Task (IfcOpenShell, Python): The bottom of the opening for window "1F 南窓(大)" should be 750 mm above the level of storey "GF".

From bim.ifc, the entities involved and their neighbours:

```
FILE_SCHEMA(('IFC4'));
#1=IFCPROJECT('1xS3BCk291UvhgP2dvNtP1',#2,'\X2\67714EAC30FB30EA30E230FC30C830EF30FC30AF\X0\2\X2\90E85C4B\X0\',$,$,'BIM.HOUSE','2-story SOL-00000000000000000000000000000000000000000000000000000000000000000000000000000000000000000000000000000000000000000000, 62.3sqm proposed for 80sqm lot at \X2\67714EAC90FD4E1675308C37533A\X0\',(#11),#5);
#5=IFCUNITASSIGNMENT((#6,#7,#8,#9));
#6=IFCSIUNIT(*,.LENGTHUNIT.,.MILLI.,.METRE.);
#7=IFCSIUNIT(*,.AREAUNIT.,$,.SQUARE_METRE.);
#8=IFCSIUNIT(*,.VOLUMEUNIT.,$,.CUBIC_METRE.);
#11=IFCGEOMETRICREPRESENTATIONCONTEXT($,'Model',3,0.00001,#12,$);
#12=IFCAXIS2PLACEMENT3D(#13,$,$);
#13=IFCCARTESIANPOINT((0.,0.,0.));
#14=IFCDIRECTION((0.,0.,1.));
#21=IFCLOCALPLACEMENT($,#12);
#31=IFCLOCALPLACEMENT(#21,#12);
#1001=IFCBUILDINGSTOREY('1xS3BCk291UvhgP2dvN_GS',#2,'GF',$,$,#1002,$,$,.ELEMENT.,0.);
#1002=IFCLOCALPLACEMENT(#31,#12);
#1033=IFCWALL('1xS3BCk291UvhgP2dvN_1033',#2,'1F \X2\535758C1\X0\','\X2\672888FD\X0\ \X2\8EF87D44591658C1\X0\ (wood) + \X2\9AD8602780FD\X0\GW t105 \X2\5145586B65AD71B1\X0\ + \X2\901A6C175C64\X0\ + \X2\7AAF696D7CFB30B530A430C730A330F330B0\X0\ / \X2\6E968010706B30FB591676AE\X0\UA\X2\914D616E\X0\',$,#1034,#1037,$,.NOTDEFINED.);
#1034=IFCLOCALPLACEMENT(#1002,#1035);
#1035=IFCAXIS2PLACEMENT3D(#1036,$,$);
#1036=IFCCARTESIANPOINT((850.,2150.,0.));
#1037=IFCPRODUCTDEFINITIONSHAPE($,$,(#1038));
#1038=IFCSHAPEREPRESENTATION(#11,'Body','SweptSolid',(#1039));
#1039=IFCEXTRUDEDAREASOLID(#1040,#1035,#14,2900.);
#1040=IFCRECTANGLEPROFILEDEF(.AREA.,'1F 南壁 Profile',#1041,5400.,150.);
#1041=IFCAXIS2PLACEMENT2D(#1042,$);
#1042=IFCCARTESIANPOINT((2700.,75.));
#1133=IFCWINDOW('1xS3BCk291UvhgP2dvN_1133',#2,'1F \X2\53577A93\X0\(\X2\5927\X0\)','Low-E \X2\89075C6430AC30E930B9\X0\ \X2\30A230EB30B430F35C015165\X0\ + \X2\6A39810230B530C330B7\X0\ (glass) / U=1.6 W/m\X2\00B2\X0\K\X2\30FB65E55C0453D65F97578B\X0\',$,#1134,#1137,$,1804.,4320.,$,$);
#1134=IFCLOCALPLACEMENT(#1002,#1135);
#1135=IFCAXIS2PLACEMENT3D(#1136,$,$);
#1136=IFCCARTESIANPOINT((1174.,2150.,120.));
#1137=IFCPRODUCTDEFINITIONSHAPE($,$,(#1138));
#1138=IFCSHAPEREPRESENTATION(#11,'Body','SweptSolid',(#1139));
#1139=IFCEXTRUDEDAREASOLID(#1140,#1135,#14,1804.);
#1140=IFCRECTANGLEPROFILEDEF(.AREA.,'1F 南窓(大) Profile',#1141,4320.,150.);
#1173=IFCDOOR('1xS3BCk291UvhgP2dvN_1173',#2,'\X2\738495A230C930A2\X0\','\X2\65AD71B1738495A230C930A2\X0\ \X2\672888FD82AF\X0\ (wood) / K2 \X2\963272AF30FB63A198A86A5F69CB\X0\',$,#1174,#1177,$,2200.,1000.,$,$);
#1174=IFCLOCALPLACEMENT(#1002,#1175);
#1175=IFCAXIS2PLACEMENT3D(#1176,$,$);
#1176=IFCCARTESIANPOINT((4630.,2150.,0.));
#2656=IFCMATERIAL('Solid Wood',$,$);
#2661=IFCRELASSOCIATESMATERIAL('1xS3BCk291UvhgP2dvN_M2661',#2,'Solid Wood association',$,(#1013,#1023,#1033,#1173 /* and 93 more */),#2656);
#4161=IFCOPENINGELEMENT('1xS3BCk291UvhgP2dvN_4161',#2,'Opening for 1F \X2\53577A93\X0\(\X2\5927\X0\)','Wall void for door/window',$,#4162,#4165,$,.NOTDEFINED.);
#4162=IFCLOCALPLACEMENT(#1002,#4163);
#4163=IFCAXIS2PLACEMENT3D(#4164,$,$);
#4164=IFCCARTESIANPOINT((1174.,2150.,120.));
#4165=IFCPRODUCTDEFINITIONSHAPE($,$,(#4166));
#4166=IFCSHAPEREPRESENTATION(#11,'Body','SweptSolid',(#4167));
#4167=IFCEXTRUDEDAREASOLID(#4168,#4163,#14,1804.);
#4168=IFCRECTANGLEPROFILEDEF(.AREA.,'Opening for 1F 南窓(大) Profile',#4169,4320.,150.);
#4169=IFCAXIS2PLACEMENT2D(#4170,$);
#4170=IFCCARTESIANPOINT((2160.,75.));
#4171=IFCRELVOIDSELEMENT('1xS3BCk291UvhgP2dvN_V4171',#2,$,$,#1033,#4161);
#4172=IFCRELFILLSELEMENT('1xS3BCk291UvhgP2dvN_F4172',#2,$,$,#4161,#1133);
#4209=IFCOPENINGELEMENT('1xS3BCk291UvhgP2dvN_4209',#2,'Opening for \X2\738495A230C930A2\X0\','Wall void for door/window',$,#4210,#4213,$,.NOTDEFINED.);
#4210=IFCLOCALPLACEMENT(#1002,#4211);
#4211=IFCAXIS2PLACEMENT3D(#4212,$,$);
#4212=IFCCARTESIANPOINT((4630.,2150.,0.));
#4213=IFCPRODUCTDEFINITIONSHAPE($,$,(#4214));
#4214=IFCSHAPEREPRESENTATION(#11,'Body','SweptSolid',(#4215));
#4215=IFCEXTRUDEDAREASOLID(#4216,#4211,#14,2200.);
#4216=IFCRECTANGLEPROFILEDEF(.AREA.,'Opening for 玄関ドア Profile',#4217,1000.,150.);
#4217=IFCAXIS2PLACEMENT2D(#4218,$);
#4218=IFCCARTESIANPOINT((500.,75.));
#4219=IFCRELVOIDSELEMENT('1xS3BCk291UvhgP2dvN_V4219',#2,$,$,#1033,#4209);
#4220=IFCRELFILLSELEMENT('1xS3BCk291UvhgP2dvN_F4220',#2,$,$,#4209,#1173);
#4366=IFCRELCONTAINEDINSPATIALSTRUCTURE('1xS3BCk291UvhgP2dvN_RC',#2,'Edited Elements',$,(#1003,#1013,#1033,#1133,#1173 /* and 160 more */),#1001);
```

```python
import numpy as np
import ifcopenshell
import ifcopenshell.api.geometry
import ifcopenshell.geom
import ifcopenshell.util.element
import ifcopenshell.util.placement
import ifcopenshell.util.shape
import ifcopenshell.util.unit

model = ifcopenshell.open("bim.ifc")
unit_scale = ifcopenshell.util.unit.calculate_unit_scale(model)

window = model.by_guid("1xS3BCk291UvhgP2dvN_1133")
opening = window.FillsVoids[0].RelatingOpeningElement
storey = ifcopenshell.util.element.get_container(window, ifc_class="IfcBuildingStorey")
level = ifcopenshell.util.placement.get_local_placement(storey.ObjectPlacement)[2, 3]

# The opening's origin need not be at the sill, so measure its lowest point.
shape = ifcopenshell.geom.create_shape(ifcopenshell.geom.settings(), opening)
bottom = ifcopenshell.util.shape.get_shape_bottom_elevation(shape, shape.geometry) / unit_scale
dz = level + 0.75 / unit_scale - bottom

shift = np.array([0.0, 0.0, dz])
# The window is not placed relative to its opening, so move both.
for product in (opening, window):
    matrix = ifcopenshell.util.placement.get_local_placement(product.ObjectPlacement)
    matrix[:3, 3] += shift
    ifcopenshell.api.geometry.edit_object_placement(model, product=product, matrix=matrix, is_si=False)

print(f"moved by {dz * unit_scale:+.3f} m")

model.write("bim_updated.ifc")
```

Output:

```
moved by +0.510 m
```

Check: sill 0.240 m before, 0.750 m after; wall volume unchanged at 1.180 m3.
